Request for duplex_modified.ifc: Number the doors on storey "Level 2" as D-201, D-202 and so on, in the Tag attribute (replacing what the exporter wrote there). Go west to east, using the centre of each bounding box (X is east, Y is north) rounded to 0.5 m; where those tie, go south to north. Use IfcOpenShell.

First a look at what the model holds.

```python
import ifcopenshell
import ifcopenshell.util.element
import ifcopenshell.util.placement

model = ifcopenshell.open("duplex_modified.ifc")
print(model.schema)
storey = next(s for s in model.by_type("IfcBuildingStorey") if s.Name == "Level 2")
doors = [e for e in ifcopenshell.util.element.get_decomposition(storey) if e.is_a("IfcDoor")]
for e in sorted(doors, key=lambda e: e.id()):
    origin = ifcopenshell.util.placement.get_local_placement(e.ObjectPlacement)[:3, 3]
    print(e.id(), e.Tag, e.Name, origin.round(2) + 0.0, sep=" | ")
```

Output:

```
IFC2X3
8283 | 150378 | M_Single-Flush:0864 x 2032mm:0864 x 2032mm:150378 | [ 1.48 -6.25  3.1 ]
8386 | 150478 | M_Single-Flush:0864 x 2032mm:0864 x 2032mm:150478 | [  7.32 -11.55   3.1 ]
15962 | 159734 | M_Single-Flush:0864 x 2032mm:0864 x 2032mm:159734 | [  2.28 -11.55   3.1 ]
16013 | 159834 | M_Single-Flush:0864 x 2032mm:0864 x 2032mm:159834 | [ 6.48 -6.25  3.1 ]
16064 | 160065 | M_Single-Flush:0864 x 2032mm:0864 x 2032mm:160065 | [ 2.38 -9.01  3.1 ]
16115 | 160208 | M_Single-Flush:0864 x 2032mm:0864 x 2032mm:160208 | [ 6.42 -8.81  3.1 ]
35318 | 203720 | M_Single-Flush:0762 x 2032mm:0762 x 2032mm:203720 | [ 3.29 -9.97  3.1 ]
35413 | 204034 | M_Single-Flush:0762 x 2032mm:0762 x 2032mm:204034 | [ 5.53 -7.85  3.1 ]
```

```python
import ifcopenshell
import ifcopenshell.geom
import ifcopenshell.util.element
import ifcopenshell.util.shape

model = ifcopenshell.open("duplex_modified.ifc")
settings = ifcopenshell.geom.settings()
settings.set("use-world-coords", True)


def centre(element):
    shape = ifcopenshell.geom.create_shape(settings, element)
    return ifcopenshell.util.shape.get_bbox_centroid(shape.geometry)


storey = next(s for s in model.by_type("IfcBuildingStorey") if s.Name == "Level 2")
doors = [e for e in ifcopenshell.util.element.get_decomposition(storey) if e.is_a("IfcDoor")]

# Insertion points can sit at a corner or the storey origin, so sort by the geometry (in metres).
centres = {e: centre(e) for e in doors}
doors.sort(key=lambda e: (round(centres[e][0] / 0.5), centres[e][1]))

for i, e in enumerate(doors, start=1):
    number = f"D-2{i:02d}"
    e.Tag = number
    print(e.id(), number)

model.write("duplex_modified_edited.ifc")
```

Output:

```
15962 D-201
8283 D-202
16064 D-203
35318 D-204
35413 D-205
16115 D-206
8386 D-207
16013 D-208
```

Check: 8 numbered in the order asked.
